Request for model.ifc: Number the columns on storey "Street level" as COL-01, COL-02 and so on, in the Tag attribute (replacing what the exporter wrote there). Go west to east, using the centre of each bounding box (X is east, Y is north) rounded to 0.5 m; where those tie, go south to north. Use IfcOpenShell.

First a look at what the model holds.

```python
import ifcopenshell
import ifcopenshell.util.element
import ifcopenshell.util.placement

model = ifcopenshell.open("model.ifc")
print(model.schema)
storey = next(s for s in model.by_type("IfcBuildingStorey") if s.Name == "Street level")
columns = [e for e in ifcopenshell.util.element.get_decomposition(storey) if e.is_a("IfcColumn")]
for e in sorted(columns, key=lambda e: e.id()):
    origin = ifcopenshell.util.placement.get_local_placement(e.ObjectPlacement)[:3, 3]
    print(e.id(), e.Tag, e.Name, origin.round(2) + 0.0, sep=" | ")
```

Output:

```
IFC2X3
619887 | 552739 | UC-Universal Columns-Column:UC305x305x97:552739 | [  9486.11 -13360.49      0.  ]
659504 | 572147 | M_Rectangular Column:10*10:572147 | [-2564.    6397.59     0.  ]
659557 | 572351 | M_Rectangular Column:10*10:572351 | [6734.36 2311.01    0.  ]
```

```python
import ifcopenshell
import ifcopenshell.geom
import ifcopenshell.util.element
import ifcopenshell.util.shape

model = ifcopenshell.open("model.ifc")
settings = ifcopenshell.geom.settings()
settings.set("use-world-coords", True)


def centre(element):
    shape = ifcopenshell.geom.create_shape(settings, element)
    return ifcopenshell.util.shape.get_bbox_centroid(shape.geometry)


storey = next(s for s in model.by_type("IfcBuildingStorey") if s.Name == "Street level")
columns = [e for e in ifcopenshell.util.element.get_decomposition(storey) if e.is_a("IfcColumn")]

# Insertion points can sit at a corner or the storey origin, so sort by the geometry (in metres).
centres = {e: centre(e) for e in columns}
columns.sort(key=lambda e: (round(centres[e][0] / 0.5), centres[e][1]))

for i, e in enumerate(columns, start=1):
    number = f"COL-{i:02d}"
    e.Tag = number
    print(e.id(), number)

model.write("model_rev.ifc")
```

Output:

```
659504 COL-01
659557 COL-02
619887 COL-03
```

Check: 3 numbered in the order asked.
